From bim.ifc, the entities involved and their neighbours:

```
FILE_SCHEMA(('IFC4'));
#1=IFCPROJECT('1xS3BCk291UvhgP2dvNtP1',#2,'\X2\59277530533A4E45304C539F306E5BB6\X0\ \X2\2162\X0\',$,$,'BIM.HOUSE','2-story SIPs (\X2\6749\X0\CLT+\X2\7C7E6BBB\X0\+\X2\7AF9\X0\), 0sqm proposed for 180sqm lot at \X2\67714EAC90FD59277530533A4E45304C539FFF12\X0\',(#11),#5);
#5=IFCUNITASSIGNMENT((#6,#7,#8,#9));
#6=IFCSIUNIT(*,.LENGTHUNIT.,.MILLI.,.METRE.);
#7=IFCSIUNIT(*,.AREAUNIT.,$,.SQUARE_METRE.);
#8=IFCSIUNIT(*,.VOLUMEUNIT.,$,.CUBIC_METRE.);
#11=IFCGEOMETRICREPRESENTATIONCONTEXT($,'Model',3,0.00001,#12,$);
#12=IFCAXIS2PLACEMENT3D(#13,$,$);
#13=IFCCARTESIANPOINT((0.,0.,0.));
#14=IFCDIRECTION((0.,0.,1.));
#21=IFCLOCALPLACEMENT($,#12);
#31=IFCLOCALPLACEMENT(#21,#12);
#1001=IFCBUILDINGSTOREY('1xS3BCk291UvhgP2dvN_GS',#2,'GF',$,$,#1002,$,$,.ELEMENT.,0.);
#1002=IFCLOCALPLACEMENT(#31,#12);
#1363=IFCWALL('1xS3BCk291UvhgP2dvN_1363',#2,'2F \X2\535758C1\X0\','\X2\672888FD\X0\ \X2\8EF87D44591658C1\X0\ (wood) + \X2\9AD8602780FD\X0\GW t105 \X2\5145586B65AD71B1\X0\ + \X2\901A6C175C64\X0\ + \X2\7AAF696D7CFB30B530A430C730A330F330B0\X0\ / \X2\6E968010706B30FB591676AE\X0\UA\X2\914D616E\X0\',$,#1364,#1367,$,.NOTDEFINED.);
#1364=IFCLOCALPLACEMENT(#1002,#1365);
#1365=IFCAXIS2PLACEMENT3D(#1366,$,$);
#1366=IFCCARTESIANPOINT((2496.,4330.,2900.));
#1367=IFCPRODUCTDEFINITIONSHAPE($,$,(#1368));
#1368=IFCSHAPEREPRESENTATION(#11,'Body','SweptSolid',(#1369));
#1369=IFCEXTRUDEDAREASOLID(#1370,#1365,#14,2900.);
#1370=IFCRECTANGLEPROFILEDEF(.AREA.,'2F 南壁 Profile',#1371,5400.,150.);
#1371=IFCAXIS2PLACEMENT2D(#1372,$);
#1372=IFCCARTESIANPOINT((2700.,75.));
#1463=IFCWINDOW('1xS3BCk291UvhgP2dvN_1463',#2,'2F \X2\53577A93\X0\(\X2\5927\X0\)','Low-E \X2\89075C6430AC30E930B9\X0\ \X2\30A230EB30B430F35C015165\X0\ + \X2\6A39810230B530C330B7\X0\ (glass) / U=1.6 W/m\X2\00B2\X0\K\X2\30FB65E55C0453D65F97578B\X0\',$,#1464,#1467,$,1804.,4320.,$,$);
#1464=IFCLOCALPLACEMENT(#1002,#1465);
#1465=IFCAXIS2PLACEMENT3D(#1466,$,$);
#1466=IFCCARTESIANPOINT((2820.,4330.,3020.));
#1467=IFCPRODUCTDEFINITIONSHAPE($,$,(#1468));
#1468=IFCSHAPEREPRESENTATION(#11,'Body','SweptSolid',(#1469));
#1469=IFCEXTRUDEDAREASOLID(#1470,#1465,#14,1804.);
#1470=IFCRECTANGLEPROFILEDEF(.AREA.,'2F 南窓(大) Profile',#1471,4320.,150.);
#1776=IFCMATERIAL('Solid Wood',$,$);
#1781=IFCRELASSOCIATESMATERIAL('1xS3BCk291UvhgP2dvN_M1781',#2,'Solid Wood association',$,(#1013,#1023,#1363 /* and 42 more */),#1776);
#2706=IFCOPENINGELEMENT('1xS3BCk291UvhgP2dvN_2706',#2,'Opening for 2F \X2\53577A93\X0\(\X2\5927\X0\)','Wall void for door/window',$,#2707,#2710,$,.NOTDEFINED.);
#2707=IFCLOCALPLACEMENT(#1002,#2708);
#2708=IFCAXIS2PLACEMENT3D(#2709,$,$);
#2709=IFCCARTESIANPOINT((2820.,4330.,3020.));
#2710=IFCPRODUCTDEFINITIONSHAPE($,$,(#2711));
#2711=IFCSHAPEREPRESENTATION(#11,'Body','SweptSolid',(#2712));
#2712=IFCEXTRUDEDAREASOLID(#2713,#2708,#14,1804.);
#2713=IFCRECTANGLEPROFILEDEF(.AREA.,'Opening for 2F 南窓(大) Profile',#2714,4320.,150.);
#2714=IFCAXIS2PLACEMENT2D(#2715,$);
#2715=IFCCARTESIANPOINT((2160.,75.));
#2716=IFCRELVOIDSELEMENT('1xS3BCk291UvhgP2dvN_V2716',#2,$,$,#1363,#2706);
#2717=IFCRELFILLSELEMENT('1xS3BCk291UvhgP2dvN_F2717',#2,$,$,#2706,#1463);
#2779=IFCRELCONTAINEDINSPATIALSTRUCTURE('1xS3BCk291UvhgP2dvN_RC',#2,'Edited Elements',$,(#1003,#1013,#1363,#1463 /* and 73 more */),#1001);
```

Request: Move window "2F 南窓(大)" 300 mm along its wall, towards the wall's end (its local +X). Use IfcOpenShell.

```python
import ifcopenshell
import ifcopenshell.api.geometry
import ifcopenshell.util.placement
import ifcopenshell.util.unit

model = ifcopenshell.open("bim.ifc")
unit_scale = ifcopenshell.util.unit.calculate_unit_scale(model)

window = model.by_guid("1xS3BCk291UvhgP2dvN_1463")
opening = window.FillsVoids[0].RelatingOpeningElement
wall = opening.VoidsElements[0].RelatingBuildingElement

wall_matrix = ifcopenshell.util.placement.get_local_placement(wall.ObjectPlacement)
shift = wall_matrix[:3, 0] * 0.3 / unit_scale
before = ifcopenshell.util.placement.get_local_placement(window.ObjectPlacement)[:3, 3].copy()

# The window is not placed relative to its opening, so move both.
for product in (opening, window):
    matrix = ifcopenshell.util.placement.get_local_placement(product.ObjectPlacement)
    matrix[:3, 3] += shift
    ifcopenshell.api.geometry.edit_object_placement(model, product=product, matrix=matrix, is_si=False)

after = ifcopenshell.util.placement.get_local_placement(window.ObjectPlacement)[:3, 3]
print("window moved by", (after - before).round(3) + 0.0)

model.write("bim_edited.ifc")
```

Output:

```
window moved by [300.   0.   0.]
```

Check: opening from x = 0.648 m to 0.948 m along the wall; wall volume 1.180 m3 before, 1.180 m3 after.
